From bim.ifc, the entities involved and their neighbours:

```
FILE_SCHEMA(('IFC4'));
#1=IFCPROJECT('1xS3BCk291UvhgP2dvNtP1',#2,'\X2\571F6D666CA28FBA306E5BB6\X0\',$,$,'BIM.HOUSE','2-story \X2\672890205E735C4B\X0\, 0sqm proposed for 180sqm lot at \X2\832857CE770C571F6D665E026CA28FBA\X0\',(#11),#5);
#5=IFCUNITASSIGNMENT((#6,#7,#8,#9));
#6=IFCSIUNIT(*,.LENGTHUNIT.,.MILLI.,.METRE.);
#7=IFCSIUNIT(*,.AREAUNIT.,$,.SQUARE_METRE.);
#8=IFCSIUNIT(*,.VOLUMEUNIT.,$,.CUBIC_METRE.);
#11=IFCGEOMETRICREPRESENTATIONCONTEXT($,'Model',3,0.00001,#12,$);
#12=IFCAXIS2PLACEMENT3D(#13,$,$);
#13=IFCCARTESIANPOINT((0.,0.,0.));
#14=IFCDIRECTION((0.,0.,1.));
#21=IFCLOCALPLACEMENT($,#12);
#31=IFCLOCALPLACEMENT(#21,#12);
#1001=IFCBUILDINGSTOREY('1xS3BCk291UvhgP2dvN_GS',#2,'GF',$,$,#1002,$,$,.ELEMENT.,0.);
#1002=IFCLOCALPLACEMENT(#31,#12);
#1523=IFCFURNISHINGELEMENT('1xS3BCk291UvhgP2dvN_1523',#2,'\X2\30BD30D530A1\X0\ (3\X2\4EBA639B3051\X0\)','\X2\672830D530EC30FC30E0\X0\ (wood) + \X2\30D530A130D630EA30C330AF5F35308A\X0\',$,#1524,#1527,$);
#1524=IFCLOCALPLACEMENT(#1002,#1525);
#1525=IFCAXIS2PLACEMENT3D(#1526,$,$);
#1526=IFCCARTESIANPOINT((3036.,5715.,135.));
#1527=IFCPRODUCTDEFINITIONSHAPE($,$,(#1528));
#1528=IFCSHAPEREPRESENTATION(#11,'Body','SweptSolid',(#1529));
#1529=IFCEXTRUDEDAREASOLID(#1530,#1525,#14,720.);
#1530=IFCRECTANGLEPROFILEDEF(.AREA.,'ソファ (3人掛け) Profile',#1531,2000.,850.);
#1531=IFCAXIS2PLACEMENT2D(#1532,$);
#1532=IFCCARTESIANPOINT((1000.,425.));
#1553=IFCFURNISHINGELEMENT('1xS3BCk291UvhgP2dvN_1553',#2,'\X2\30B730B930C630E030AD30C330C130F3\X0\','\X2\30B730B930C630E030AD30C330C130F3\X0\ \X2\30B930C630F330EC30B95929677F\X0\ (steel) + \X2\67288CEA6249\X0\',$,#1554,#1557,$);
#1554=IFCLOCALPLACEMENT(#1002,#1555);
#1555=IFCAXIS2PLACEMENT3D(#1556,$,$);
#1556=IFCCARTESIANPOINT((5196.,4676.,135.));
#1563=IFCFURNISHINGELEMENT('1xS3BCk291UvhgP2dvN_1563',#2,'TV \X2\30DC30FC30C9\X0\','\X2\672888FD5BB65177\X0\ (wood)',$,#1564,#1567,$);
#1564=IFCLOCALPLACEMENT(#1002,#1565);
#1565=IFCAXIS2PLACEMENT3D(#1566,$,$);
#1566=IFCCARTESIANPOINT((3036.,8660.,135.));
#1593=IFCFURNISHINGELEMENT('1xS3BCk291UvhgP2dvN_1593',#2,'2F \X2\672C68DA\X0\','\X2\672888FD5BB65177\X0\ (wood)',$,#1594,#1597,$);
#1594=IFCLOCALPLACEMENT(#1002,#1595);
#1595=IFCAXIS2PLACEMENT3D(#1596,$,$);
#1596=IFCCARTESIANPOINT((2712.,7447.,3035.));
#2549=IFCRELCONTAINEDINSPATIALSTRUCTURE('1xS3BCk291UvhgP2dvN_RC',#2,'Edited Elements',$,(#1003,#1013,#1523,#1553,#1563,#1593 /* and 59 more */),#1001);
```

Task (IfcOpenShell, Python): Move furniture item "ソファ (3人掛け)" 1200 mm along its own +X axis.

```python
import ifcopenshell
import ifcopenshell.api.geometry
import ifcopenshell.util.placement
import ifcopenshell.util.unit

model = ifcopenshell.open("bim.ifc")
unit_scale = ifcopenshell.util.unit.calculate_unit_scale(model)

item = model.by_guid("1xS3BCk291UvhgP2dvN_1523")
matrix = ifcopenshell.util.placement.get_local_placement(item.ObjectPlacement)
matrix[:3, 3] += matrix[:3, 0] * 1.2 / unit_scale
ifcopenshell.api.geometry.edit_object_placement(model, product=item, matrix=matrix, is_si=False)

print(ifcopenshell.util.placement.get_local_placement(item.ObjectPlacement).round(3) + 0.0)

model.write("bim_edited.ifc")
```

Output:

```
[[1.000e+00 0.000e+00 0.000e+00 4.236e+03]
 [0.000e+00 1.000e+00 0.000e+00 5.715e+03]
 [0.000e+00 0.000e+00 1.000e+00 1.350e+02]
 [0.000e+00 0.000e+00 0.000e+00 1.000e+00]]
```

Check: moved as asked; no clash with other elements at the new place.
